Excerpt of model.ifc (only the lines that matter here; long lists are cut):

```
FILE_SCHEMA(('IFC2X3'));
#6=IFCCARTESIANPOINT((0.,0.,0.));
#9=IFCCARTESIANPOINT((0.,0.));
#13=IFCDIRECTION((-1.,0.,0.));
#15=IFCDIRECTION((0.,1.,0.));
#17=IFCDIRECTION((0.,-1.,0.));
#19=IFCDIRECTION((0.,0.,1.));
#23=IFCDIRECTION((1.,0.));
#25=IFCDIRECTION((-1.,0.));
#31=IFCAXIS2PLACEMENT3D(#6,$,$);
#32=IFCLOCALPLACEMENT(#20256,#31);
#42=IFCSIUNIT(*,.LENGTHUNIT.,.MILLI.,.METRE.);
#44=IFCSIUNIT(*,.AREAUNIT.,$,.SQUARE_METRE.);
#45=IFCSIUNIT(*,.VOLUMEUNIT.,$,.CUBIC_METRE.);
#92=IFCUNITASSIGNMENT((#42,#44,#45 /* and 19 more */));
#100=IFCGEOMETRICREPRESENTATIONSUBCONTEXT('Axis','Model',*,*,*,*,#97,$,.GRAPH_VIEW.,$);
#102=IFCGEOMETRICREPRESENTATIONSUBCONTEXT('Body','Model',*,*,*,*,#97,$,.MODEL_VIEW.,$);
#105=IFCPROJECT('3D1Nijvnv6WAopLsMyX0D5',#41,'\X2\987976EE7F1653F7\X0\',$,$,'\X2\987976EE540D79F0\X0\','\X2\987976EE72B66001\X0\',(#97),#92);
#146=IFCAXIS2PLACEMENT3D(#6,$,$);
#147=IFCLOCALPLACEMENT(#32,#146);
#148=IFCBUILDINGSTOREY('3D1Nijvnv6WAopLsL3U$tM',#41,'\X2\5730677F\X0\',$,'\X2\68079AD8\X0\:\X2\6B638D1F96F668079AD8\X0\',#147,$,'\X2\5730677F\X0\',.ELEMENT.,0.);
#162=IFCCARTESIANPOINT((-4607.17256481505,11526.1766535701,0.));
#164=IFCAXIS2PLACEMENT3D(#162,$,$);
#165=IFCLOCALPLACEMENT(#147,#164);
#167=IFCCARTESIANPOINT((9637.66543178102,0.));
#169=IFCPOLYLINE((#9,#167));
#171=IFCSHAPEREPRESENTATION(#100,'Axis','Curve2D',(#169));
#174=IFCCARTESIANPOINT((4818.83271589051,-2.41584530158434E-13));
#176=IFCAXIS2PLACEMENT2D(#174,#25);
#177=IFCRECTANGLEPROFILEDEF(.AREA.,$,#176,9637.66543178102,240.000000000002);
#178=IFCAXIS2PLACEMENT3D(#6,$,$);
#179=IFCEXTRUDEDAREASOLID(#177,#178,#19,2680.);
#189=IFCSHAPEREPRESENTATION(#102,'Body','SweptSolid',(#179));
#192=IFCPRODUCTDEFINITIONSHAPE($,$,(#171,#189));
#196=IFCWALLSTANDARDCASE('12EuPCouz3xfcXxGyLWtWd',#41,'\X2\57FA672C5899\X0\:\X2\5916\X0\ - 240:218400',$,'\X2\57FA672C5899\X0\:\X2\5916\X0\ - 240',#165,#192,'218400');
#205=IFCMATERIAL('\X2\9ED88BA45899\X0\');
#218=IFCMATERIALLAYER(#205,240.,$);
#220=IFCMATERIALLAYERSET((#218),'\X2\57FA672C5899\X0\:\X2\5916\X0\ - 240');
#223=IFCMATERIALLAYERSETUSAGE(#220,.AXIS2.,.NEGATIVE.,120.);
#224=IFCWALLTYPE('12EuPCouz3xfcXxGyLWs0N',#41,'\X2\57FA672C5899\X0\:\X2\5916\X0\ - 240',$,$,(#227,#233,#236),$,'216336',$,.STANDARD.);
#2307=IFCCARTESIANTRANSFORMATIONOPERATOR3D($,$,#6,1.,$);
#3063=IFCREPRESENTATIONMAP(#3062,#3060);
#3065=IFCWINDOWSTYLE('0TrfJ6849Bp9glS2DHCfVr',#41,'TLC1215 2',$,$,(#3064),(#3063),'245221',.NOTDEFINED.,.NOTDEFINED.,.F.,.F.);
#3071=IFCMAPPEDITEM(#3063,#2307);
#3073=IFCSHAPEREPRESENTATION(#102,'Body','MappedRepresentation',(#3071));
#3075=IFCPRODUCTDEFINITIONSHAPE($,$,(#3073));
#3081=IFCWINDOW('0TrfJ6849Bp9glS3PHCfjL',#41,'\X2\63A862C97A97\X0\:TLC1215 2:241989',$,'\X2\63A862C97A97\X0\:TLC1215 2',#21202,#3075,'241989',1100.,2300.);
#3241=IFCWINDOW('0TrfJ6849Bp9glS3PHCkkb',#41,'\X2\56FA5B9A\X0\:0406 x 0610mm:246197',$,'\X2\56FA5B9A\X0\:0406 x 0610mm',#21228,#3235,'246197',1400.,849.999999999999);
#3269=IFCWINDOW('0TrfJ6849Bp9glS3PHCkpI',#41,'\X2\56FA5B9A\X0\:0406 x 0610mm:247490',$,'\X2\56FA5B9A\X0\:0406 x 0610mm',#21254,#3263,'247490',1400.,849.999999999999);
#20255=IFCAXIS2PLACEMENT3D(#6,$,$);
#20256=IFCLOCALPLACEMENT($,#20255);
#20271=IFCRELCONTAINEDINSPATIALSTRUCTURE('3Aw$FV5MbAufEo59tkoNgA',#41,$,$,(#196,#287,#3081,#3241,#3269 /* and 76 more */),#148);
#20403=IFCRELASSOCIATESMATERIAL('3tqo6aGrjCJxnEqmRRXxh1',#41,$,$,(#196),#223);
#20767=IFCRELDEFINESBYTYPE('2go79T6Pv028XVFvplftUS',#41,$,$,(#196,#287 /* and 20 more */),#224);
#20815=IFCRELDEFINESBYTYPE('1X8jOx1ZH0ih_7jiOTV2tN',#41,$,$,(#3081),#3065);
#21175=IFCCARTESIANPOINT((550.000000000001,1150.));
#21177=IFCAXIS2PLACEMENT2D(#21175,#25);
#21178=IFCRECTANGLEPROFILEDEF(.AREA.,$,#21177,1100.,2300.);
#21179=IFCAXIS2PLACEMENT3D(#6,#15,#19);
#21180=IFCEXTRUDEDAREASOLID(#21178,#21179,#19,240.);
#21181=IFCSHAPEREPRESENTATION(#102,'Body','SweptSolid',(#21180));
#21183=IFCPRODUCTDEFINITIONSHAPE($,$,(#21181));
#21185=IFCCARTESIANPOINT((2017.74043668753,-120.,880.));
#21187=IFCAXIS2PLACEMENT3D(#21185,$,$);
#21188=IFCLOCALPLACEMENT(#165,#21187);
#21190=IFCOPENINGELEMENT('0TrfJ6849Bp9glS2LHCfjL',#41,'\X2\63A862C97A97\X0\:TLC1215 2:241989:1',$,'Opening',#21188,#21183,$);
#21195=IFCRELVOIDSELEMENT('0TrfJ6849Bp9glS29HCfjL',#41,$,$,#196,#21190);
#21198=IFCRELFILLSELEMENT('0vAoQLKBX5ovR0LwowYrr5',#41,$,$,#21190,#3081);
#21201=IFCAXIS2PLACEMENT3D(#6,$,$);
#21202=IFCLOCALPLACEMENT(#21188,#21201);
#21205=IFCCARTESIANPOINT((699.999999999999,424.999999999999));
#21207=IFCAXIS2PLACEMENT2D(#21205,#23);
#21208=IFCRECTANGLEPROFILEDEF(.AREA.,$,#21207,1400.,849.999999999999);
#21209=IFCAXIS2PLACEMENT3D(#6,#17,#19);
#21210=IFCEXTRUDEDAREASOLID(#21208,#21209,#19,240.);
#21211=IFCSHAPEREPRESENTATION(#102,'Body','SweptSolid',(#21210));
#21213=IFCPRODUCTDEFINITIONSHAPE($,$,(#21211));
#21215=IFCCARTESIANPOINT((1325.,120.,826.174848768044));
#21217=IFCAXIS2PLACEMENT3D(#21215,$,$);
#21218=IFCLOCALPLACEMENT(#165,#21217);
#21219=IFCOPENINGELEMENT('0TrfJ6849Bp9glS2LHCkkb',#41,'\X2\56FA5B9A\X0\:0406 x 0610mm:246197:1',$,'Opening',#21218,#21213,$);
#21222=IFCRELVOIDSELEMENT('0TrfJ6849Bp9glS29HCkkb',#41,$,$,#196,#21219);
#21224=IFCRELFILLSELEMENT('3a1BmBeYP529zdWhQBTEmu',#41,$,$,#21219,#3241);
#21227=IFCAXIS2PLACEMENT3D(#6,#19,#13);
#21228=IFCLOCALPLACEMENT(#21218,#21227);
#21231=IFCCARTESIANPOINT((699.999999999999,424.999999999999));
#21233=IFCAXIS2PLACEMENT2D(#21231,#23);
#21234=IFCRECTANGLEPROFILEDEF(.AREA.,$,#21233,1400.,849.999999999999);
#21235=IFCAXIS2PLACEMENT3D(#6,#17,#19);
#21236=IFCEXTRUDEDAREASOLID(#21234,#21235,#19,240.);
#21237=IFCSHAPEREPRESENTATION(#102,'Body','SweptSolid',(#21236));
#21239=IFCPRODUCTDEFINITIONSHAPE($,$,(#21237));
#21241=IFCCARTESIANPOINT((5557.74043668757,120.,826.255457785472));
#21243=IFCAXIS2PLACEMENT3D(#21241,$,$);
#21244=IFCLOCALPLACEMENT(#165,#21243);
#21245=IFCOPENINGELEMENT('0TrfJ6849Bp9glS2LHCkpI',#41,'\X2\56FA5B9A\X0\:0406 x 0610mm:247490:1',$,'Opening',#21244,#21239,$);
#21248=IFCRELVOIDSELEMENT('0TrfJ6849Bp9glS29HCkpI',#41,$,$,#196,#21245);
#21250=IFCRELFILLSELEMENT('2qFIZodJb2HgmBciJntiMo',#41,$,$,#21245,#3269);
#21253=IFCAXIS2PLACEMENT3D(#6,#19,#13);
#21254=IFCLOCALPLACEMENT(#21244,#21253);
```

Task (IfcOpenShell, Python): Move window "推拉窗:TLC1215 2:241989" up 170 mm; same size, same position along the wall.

```python
import numpy as np
import ifcopenshell
import ifcopenshell.api.geometry
import ifcopenshell.util.placement
import ifcopenshell.util.unit

model = ifcopenshell.open("model.ifc")
unit_scale = ifcopenshell.util.unit.calculate_unit_scale(model)

window = model.by_id(3081)
opening = window.FillsVoids[0].RelatingOpeningElement
dz = 0.17 / unit_scale

shift = np.array([0.0, 0.0, dz])
# The window is placed relative to its opening, so it follows when the opening moves.
matrix = ifcopenshell.util.placement.get_local_placement(opening.ObjectPlacement)
matrix[:3, 3] += shift
ifcopenshell.api.geometry.edit_object_placement(
    model, product=opening, matrix=matrix, is_si=False, should_transform_children=True
)

print(f"moved by {dz * unit_scale:+.3f} m")

model.write("model-out.ifc")
```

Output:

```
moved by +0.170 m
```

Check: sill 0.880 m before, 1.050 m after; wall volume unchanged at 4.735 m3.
